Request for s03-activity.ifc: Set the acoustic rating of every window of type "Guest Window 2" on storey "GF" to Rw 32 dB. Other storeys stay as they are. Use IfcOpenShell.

First a look at what the model holds.

```python
import ifcopenshell
import ifcopenshell.util.element

model = ifcopenshell.open("s03-activity.ifc")
print(model.schema)
storey = next(s for s in model.by_type("IfcBuildingStorey") if s.Name == "GF")
windows = [e for e in ifcopenshell.util.element.get_decomposition(storey) if e.is_a("IfcWindow")]
seen = {}
for e in windows:
    element_type = ifcopenshell.util.element.get_type(e)
    key = (element_type.Name if element_type != e and element_type else None, ifcopenshell.util.element.get_pset(e, "Pset_WindowCommon", "AcousticRating"))
    seen[key] = seen.get(key, 0) + 1
for (name, value), count in sorted(seen.items(), key=str):
    print(count, "x", name, "|", value)
```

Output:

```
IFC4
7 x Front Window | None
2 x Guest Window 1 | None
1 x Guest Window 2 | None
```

```python
import ifcopenshell
import ifcopenshell.api.pset
import ifcopenshell.util.element

model = ifcopenshell.open("s03-activity.ifc")

storey = next(s for s in model.by_type("IfcBuildingStorey") if s.Name == "GF")
windows = [e for e in ifcopenshell.util.element.get_decomposition(storey) if e.is_a("IfcWindow")]

count = 0
for e in windows:
    element_type = ifcopenshell.util.element.get_type(e)
    if element_type in (None, e) or element_type.Name != "Guest Window 2":
        continue
    # add_pset returns the element's existing set when there is one.
    pset = ifcopenshell.api.pset.add_pset(model, product=e, name="Pset_WindowCommon")
    ifcopenshell.api.pset.edit_pset(model, pset=pset, properties={"AcousticRating": "Rw 32 dB"})
    count += 1

print(count, "windows updated")

model.write("s03-activity_v2.ifc")
```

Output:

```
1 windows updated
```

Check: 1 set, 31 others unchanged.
